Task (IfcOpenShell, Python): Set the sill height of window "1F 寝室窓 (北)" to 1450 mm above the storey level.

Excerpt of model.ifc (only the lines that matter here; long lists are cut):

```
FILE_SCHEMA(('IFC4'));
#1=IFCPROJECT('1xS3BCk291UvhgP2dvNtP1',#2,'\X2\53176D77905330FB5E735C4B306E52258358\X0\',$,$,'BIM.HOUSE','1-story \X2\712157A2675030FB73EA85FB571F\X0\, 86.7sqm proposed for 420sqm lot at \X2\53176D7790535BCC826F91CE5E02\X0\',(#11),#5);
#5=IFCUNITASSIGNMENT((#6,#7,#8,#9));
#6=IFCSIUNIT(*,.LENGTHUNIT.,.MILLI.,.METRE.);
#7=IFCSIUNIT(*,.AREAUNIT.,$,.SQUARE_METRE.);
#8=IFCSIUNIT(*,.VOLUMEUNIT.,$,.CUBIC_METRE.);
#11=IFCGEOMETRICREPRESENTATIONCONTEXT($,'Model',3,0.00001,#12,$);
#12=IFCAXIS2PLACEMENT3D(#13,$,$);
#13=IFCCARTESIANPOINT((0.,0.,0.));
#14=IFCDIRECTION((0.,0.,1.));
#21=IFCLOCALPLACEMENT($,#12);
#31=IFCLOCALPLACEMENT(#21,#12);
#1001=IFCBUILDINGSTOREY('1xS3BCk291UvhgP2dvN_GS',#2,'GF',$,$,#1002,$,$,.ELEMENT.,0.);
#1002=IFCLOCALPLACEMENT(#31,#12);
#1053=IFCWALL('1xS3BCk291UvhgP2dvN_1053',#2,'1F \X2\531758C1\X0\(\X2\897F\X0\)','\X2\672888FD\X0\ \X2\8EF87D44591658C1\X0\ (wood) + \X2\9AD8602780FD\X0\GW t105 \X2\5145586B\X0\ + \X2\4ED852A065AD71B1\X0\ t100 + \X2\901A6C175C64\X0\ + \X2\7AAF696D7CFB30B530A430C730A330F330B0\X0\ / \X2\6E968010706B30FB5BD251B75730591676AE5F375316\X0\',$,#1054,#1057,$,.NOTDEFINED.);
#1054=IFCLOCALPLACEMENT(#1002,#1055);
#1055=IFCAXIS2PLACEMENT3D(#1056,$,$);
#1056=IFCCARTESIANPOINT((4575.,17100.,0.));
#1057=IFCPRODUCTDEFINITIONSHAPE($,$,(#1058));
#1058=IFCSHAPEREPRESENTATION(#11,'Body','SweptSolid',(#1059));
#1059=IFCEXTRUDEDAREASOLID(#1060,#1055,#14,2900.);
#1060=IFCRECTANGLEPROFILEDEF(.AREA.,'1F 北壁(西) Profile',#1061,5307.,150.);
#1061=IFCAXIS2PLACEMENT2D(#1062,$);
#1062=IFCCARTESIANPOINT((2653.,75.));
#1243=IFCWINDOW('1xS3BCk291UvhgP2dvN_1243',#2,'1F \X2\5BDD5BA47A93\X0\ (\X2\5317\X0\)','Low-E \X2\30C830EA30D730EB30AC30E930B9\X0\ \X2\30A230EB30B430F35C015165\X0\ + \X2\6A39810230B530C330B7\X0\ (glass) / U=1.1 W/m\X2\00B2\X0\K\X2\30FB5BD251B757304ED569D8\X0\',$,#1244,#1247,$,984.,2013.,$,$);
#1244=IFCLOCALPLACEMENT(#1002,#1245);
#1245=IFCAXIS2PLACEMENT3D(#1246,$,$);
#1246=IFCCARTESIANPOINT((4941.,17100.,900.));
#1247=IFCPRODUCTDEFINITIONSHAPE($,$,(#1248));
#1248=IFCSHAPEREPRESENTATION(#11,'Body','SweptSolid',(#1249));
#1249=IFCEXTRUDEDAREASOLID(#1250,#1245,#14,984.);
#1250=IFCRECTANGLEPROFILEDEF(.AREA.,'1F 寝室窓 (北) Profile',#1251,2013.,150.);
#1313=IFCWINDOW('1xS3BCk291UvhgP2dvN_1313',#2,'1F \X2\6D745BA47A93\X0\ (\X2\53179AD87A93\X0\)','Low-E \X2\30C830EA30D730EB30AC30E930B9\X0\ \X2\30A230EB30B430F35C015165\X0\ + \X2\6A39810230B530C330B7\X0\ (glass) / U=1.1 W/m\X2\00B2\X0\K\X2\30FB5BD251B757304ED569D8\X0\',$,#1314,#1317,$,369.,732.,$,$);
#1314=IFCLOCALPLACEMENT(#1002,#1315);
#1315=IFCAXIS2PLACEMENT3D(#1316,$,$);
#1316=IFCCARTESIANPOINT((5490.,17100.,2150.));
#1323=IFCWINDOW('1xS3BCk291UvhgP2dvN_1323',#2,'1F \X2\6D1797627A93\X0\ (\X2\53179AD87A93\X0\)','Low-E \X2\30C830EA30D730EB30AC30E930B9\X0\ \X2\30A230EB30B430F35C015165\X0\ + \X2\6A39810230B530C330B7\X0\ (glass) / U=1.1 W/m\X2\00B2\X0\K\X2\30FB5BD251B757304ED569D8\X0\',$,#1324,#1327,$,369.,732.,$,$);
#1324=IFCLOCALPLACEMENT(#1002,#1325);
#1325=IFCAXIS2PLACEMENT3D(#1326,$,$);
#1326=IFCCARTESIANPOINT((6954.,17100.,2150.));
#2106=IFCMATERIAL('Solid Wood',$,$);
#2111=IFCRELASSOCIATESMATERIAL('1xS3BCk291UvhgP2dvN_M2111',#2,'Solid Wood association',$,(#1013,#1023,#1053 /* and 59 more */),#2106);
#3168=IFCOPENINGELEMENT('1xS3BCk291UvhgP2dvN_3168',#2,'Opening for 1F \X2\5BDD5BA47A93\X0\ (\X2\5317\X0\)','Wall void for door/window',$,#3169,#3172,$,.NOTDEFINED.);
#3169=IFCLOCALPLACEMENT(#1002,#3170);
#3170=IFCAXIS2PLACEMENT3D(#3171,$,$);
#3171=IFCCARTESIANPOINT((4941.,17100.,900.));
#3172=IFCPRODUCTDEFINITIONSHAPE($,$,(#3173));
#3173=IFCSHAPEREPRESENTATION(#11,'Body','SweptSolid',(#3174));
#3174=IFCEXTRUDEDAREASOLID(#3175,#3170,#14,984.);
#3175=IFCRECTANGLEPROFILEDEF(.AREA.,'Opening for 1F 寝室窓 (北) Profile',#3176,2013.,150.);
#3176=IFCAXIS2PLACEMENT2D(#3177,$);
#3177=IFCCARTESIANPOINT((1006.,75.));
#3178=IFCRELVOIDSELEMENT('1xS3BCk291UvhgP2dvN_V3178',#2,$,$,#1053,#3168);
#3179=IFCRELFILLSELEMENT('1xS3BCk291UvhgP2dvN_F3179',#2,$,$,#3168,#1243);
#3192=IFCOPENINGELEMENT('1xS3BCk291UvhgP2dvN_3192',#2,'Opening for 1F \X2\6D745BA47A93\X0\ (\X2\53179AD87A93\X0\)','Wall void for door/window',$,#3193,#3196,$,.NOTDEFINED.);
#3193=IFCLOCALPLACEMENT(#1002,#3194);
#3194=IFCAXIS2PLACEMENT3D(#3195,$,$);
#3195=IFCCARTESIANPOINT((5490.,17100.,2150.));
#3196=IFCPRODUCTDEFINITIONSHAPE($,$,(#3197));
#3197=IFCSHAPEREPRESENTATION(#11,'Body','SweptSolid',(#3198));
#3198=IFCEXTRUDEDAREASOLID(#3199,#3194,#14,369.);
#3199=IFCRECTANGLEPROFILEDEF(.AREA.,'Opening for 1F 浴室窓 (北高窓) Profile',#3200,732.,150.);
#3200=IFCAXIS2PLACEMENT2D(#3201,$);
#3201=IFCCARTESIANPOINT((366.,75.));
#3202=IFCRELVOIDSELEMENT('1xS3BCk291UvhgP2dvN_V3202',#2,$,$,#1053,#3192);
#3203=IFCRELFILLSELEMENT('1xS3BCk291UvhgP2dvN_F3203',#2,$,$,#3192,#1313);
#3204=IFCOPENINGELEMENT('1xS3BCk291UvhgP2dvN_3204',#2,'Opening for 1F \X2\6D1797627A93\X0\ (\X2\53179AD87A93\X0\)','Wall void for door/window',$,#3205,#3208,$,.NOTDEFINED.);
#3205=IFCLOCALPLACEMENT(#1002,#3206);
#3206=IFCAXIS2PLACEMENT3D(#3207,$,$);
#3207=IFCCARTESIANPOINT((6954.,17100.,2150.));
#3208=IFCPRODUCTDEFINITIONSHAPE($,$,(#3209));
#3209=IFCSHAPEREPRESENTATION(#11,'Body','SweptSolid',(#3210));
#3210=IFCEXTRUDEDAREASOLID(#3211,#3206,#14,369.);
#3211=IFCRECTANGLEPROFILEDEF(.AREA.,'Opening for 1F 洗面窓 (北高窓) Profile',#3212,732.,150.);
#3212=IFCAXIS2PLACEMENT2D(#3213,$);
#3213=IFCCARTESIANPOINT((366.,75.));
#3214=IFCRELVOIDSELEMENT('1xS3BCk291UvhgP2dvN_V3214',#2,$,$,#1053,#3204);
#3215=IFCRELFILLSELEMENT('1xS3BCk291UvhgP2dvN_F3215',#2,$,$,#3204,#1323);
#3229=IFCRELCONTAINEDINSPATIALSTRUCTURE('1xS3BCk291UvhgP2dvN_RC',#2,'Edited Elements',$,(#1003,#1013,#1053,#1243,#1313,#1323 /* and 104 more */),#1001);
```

```python
import numpy as np
import ifcopenshell
import ifcopenshell.api.geometry
import ifcopenshell.geom
import ifcopenshell.util.element
import ifcopenshell.util.placement
import ifcopenshell.util.shape
import ifcopenshell.util.unit

model = ifcopenshell.open("model.ifc")
unit_scale = ifcopenshell.util.unit.calculate_unit_scale(model)

window = model.by_id(1243)
opening = window.FillsVoids[0].RelatingOpeningElement
storey = ifcopenshell.util.element.get_container(window, ifc_class="IfcBuildingStorey")
level = ifcopenshell.util.placement.get_local_placement(storey.ObjectPlacement)[2, 3]

# The opening's origin need not be at the sill, so measure its lowest point.
shape = ifcopenshell.geom.create_shape(ifcopenshell.geom.settings(), opening)
bottom = ifcopenshell.util.shape.get_shape_bottom_elevation(shape, shape.geometry) / unit_scale
dz = level + 1.45 / unit_scale - bottom

shift = np.array([0.0, 0.0, dz])
# The window is not placed relative to its opening, so move both.
for product in (opening, window):
    matrix = ifcopenshell.util.placement.get_local_placement(product.ObjectPlacement)
    matrix[:3, 3] += shift
    ifcopenshell.api.geometry.edit_object_placement(model, product=product, matrix=matrix, is_si=False)

print(f"moved by {dz * unit_scale:+.3f} m")

model.write("model_v2.ifc")
```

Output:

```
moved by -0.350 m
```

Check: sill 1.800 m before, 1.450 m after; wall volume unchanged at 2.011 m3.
